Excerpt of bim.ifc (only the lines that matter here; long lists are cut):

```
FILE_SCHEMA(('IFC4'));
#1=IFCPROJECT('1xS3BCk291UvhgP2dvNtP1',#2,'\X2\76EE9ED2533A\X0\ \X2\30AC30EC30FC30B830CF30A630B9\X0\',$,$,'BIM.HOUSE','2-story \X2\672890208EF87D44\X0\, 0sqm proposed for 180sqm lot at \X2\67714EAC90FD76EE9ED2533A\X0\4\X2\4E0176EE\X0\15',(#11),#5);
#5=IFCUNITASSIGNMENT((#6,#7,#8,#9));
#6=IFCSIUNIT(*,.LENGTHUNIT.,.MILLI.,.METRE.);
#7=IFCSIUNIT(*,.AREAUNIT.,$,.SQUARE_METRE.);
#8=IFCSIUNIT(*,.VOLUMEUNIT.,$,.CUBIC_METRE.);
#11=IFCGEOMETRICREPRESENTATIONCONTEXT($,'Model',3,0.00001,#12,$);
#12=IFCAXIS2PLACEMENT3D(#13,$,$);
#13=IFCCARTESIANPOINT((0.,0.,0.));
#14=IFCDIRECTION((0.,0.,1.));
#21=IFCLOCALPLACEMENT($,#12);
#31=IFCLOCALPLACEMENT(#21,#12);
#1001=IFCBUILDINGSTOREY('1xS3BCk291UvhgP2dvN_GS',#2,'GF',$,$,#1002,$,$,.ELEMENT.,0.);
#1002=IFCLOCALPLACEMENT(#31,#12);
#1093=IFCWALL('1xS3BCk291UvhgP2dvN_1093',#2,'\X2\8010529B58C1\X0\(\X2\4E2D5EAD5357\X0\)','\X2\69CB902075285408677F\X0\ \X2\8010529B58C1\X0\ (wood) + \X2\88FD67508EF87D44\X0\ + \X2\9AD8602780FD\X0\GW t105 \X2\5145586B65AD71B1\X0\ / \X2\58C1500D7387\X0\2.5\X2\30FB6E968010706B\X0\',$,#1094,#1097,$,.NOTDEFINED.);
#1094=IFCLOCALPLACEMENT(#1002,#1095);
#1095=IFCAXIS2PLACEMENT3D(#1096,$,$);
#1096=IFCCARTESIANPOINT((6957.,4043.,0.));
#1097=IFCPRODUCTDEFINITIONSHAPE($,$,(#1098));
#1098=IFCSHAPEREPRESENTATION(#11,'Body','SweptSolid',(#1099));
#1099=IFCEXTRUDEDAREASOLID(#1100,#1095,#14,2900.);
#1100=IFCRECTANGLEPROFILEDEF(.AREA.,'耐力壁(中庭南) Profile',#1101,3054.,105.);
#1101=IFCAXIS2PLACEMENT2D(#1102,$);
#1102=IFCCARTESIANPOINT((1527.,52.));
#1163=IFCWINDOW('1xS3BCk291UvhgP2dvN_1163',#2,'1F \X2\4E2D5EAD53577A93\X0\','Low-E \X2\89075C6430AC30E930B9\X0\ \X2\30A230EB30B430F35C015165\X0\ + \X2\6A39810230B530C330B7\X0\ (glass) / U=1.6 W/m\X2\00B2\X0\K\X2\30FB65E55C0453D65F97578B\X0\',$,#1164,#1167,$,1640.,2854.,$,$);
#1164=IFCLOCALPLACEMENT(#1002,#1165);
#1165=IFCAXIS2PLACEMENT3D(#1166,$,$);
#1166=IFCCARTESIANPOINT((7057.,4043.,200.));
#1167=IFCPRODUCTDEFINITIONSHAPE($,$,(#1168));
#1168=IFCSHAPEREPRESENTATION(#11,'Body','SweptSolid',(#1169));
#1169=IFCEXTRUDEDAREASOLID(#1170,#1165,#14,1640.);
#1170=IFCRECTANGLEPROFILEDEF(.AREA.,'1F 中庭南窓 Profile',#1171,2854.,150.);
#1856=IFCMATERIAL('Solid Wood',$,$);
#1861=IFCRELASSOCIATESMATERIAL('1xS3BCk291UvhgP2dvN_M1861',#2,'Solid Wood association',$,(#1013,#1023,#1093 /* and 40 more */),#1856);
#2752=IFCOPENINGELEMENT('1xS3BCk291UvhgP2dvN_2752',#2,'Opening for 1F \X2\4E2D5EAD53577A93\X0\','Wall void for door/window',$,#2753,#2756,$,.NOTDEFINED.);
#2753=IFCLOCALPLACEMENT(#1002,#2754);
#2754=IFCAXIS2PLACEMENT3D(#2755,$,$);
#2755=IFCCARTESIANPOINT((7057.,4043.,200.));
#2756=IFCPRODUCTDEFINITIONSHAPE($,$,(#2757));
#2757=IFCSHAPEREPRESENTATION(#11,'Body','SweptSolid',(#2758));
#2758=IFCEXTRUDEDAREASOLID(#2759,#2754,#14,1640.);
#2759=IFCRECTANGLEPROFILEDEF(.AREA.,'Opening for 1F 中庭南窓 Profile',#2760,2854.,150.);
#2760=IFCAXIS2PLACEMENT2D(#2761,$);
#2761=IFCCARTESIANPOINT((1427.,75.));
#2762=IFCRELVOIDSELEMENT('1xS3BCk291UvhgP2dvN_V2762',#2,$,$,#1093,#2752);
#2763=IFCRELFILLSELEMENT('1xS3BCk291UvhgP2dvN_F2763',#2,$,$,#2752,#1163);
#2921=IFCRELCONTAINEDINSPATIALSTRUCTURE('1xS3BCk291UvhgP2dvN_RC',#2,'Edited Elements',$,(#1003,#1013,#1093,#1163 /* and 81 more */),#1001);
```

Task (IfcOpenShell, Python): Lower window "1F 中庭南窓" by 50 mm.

```python
import numpy as np
import ifcopenshell
import ifcopenshell.api.geometry
import ifcopenshell.util.placement
import ifcopenshell.util.unit

model = ifcopenshell.open("bim.ifc")
unit_scale = ifcopenshell.util.unit.calculate_unit_scale(model)

window = model.by_guid("1xS3BCk291UvhgP2dvN_1163")
opening = window.FillsVoids[0].RelatingOpeningElement
dz = -0.05 / unit_scale

shift = np.array([0.0, 0.0, dz])
# The window is not placed relative to its opening, so move both.
for product in (opening, window):
    matrix = ifcopenshell.util.placement.get_local_placement(product.ObjectPlacement)
    matrix[:3, 3] += shift
    ifcopenshell.api.geometry.edit_object_placement(model, product=product, matrix=matrix, is_si=False)

print(f"moved by {dz * unit_scale:+.3f} m")

model.write("bim_rev.ifc")
```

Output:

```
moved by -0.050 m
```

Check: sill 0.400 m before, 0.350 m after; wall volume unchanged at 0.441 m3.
